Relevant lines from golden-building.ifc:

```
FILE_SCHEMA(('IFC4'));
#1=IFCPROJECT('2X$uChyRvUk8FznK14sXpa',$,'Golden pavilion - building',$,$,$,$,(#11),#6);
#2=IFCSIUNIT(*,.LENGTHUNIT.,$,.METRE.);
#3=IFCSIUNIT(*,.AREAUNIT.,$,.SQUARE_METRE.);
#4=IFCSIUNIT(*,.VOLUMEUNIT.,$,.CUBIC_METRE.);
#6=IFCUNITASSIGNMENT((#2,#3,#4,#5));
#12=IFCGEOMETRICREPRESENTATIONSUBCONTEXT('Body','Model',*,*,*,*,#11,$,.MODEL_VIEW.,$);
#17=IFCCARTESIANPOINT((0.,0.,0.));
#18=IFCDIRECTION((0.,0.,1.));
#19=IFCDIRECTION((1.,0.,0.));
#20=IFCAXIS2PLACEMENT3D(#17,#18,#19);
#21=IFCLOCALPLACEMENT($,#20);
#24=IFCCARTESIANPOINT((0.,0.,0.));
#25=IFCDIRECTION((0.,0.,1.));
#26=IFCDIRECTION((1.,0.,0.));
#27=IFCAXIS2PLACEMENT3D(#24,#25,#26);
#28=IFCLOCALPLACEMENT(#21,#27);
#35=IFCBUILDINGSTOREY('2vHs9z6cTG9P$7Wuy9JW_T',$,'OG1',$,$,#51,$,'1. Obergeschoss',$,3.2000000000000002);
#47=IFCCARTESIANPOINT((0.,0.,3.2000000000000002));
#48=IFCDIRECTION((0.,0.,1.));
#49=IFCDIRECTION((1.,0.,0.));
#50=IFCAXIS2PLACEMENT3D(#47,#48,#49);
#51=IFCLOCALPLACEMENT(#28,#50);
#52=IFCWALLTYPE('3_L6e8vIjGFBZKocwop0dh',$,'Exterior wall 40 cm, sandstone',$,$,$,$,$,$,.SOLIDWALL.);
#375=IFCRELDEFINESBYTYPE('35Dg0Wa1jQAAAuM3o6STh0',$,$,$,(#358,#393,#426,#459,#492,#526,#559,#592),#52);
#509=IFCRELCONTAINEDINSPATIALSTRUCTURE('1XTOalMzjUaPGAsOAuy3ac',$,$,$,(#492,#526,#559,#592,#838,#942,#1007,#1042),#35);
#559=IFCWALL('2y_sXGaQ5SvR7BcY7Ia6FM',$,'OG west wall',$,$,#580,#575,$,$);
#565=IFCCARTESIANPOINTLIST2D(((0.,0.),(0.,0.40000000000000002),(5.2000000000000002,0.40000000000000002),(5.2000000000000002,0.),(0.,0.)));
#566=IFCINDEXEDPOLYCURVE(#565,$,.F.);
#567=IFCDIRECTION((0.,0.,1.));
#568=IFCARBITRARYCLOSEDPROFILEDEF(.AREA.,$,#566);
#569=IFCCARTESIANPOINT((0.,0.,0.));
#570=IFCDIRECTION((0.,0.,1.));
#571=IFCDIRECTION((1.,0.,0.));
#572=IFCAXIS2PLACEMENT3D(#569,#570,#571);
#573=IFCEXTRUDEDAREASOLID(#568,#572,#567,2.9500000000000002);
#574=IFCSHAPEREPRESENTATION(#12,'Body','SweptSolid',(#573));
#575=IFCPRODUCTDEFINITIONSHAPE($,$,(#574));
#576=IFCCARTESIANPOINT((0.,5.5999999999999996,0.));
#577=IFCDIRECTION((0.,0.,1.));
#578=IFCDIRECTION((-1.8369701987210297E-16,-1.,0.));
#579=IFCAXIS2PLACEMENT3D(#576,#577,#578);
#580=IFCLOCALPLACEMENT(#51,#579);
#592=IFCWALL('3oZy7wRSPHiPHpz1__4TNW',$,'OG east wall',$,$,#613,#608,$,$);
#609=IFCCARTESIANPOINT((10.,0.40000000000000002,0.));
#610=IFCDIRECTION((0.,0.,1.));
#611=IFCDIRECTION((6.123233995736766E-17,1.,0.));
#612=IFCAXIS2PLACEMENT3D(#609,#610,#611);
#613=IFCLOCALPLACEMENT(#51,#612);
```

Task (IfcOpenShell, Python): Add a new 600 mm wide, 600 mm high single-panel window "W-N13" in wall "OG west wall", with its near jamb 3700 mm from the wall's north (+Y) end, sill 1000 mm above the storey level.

```python
import numpy as np
import ifcopenshell
import ifcopenshell.api.feature
import ifcopenshell.api.geometry
import ifcopenshell.api.root
import ifcopenshell.api.spatial
import ifcopenshell.geom
import ifcopenshell.util.element
import ifcopenshell.util.placement
import ifcopenshell.util.representation
import ifcopenshell.util.shape
import ifcopenshell.util.unit

model = ifcopenshell.open("golden-building.ifc")
unit_scale = ifcopenshell.util.unit.calculate_unit_scale(model)
settings = ifcopenshell.geom.settings()


def volume(element):
    """Net volume in cubic metres, openings subtracted."""
    shape = ifcopenshell.geom.create_shape(settings, element)
    return ifcopenshell.util.shape.get_volume(shape.geometry)


wall = model.by_id(559)
storey = ifcopenshell.util.element.get_container(wall, ifc_class="IfcBuildingStorey")
context = ifcopenshell.util.representation.get_context(model, "Model", "Body", "MODEL_VIEW")
before = volume(wall)

width, height, from_end, sill = 0.6, 0.6, 3.7, 1  # metres

# The wall runs along its own X axis, and the end named is its -X end.
wall_shape = ifcopenshell.geom.create_shape(settings, wall)
x, y, z = ifcopenshell.util.shape.get_vertices(wall_shape.geometry).T
start = x.min() + from_end
face, thickness = float(y.min()), float(y.max() - y.min())
wall_matrix = ifcopenshell.util.placement.get_local_placement(wall.ObjectPlacement)
level = ifcopenshell.util.placement.get_local_placement(storey.ObjectPlacement)[2, 3]


def in_wall(x, y):
    """Placement at x, y metres in the wall's axes, at sill height."""
    matrix = wall_matrix.copy()
    matrix[:, 3] = wall_matrix @ np.array([x / unit_scale, y / unit_scale, 0.0, 1.0])
    matrix[2, 3] = level + sill / unit_scale
    return matrix


# Opening: a box that overshoots both wall faces by 50 mm.
opening = ifcopenshell.api.root.create_entity(model, ifc_class="IfcOpeningElement", predefined_type="OPENING")
box = ifcopenshell.api.geometry.add_wall_representation(
    model, context=context, length=width, height=height, thickness=thickness + 0.1
)
ifcopenshell.api.geometry.assign_representation(model, product=opening, representation=box)
ifcopenshell.api.geometry.edit_object_placement(model, product=opening, matrix=in_wall(start, face - 0.05), is_si=False)
ifcopenshell.api.feature.add_feature(model, feature=opening, element=wall)

window = ifcopenshell.api.root.create_entity(model, ifc_class="IfcWindow", name="W-N13", predefined_type="WINDOW")
window.OverallWidth, window.OverallHeight = width / unit_scale, height / unit_scale
window.PartitioningType = "SINGLE_PANEL"
body = ifcopenshell.api.geometry.add_window_representation(
    model,
    context=context,
    overall_width=window.OverallWidth,
    overall_height=window.OverallHeight,
    partition_type="SINGLE_PANEL",
)
ifcopenshell.api.geometry.assign_representation(model, product=window, representation=body)
ifcopenshell.api.spatial.assign_container(model, products=[window], relating_structure=storey)
ifcopenshell.api.feature.add_filling(model, opening=opening, element=window)

# Centre the window in the wall's thickness.
ifcopenshell.api.geometry.edit_object_placement(model, product=window, matrix=in_wall(start, face), is_si=False)
window_shape = ifcopenshell.geom.create_shape(settings, window)
depth = ifcopenshell.util.shape.get_vertices(window_shape.geometry)[:, 1]
offset = face + thickness / 2 - (depth.min() + depth.max()) / 2
ifcopenshell.api.geometry.edit_object_placement(model, product=window, matrix=in_wall(start, offset), is_si=False)

after = volume(wall)

print(f"wall volume {before:.3f} -> {after:.3f} m3")

model.write("golden-building_edited.ifc")
```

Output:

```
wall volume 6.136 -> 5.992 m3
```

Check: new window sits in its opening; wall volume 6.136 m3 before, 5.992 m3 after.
